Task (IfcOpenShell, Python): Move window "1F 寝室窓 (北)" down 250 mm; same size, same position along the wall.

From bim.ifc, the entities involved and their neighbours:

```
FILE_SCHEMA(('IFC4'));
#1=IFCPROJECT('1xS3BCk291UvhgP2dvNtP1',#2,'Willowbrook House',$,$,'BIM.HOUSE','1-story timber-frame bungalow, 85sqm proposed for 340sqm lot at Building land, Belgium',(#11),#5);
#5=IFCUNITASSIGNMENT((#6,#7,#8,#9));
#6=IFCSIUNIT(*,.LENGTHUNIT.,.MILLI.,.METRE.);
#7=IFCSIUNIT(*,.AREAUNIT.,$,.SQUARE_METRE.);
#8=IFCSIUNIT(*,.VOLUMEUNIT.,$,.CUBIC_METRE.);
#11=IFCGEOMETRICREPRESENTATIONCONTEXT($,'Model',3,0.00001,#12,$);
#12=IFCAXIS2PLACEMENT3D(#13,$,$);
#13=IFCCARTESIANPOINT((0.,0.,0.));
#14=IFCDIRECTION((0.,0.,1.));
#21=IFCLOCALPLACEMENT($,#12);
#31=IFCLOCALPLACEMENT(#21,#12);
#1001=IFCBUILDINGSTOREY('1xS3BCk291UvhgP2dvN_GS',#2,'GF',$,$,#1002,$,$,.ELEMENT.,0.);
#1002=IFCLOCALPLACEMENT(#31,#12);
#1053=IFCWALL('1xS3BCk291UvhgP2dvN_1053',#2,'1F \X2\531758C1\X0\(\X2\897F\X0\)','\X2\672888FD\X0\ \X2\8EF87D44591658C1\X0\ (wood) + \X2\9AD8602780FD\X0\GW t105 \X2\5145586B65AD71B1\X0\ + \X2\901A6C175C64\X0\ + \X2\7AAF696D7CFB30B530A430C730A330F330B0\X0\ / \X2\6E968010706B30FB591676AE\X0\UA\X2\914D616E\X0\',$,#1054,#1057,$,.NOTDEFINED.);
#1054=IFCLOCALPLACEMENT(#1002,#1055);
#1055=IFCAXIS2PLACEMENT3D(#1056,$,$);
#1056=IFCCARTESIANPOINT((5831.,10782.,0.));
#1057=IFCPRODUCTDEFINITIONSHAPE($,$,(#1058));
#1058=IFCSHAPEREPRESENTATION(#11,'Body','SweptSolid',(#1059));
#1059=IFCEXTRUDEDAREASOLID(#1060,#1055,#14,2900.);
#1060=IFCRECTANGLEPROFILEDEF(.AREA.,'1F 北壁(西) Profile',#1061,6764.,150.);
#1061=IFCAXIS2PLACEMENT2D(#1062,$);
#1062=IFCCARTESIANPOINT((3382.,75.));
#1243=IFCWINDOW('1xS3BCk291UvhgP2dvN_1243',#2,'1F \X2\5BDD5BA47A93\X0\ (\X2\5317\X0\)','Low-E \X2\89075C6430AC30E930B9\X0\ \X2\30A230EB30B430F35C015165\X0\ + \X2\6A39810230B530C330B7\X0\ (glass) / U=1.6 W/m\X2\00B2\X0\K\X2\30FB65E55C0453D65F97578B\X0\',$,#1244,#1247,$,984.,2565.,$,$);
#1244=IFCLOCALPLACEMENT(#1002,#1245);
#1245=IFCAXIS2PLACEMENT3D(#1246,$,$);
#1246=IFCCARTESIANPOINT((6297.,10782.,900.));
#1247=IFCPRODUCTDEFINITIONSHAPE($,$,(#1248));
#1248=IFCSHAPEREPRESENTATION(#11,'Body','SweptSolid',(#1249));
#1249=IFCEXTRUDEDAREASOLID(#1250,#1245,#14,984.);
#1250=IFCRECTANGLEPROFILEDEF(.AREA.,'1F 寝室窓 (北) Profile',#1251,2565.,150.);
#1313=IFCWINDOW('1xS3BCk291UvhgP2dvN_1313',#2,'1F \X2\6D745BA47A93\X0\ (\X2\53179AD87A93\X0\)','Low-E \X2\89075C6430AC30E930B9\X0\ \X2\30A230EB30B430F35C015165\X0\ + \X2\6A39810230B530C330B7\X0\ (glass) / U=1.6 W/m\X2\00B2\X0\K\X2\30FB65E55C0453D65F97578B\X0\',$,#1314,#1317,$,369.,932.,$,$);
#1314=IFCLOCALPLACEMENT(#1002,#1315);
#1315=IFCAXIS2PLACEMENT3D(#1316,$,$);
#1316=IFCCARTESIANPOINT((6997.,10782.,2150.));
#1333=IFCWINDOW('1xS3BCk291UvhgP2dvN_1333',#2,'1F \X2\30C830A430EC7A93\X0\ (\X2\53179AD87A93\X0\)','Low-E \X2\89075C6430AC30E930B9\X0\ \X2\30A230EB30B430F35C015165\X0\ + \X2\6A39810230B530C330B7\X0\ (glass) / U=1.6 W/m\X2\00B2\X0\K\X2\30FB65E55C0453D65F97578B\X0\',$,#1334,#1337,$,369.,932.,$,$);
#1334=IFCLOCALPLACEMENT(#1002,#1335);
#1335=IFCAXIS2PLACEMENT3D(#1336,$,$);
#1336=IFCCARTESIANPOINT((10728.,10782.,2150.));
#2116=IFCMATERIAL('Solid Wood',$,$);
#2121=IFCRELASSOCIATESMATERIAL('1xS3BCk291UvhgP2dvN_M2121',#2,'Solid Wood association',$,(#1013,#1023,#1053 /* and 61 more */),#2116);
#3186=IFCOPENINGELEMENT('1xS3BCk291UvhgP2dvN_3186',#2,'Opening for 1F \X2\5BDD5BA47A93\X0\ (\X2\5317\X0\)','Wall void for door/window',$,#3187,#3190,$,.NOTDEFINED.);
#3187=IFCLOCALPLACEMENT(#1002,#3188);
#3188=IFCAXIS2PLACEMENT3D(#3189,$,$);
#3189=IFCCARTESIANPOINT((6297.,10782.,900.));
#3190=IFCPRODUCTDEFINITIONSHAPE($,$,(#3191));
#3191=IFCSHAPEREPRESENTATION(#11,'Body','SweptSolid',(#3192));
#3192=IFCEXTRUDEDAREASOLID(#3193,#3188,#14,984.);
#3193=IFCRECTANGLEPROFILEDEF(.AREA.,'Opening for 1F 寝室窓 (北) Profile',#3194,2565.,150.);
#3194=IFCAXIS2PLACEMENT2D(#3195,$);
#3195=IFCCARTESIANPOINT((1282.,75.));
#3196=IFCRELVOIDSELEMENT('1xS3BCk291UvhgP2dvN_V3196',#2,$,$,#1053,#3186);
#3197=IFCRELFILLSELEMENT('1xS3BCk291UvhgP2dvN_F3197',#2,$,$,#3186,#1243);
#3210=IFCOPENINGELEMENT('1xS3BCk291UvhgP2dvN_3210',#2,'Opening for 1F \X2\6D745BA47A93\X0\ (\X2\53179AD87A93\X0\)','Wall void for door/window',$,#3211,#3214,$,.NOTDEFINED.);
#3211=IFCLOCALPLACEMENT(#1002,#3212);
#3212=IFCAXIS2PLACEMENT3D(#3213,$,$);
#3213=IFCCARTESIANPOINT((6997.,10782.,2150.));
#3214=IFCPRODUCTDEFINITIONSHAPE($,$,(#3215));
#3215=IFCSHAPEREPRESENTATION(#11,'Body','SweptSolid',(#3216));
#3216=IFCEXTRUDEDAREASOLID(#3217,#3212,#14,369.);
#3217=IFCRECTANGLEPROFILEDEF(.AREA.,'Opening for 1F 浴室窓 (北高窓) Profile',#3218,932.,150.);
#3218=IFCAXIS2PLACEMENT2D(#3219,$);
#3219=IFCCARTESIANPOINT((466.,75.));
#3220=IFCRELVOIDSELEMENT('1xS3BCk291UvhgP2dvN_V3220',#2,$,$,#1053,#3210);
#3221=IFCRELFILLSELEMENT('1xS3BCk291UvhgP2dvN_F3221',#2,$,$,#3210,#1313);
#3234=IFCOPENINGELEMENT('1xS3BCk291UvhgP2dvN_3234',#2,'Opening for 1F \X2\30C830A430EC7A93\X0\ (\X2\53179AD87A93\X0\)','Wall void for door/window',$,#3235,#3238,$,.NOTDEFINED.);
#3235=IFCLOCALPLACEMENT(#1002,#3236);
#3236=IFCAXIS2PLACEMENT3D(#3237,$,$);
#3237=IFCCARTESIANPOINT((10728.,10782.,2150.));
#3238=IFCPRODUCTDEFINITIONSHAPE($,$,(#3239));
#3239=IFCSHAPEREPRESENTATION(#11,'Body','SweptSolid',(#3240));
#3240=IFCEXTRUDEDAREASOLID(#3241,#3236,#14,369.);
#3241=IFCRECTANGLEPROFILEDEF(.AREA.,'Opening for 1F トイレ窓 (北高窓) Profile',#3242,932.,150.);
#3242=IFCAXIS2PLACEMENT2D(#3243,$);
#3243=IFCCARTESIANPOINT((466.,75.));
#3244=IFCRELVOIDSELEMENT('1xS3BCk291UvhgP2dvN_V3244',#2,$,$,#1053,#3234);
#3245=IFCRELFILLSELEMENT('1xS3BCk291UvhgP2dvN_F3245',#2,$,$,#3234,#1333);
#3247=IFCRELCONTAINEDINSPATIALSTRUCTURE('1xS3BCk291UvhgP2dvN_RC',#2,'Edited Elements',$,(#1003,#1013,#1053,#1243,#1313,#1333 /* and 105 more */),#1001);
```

```python
import numpy as np
import ifcopenshell
import ifcopenshell.api.geometry
import ifcopenshell.util.placement
import ifcopenshell.util.unit

model = ifcopenshell.open("bim.ifc")
unit_scale = ifcopenshell.util.unit.calculate_unit_scale(model)

window = model.by_guid("1xS3BCk291UvhgP2dvN_1243")
opening = window.FillsVoids[0].RelatingOpeningElement
dz = -0.25 / unit_scale

shift = np.array([0.0, 0.0, dz])
# The window is not placed relative to its opening, so move both.
for product in (opening, window):
    matrix = ifcopenshell.util.placement.get_local_placement(product.ObjectPlacement)
    matrix[:3, 3] += shift
    ifcopenshell.api.geometry.edit_object_placement(model, product=product, matrix=matrix, is_si=False)

print(f"moved by {dz * unit_scale:+.3f} m")

model.write("bim-out.ifc")
```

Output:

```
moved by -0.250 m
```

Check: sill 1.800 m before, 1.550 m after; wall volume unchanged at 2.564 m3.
